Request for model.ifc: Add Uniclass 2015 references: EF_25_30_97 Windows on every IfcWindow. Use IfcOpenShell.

First a look at what the model holds.

```python
import ifcopenshell

model = ifcopenshell.open("model.ifc")
print(model.schema)
print("classifications:", [c.Name for c in model.by_type("IfcClassification")])
for ifc_class in ("IfcDoor", "IfcRoof", "IfcStair", "IfcWall", "IfcWindow"):
    print(ifc_class, len(model.by_type(ifc_class)))
```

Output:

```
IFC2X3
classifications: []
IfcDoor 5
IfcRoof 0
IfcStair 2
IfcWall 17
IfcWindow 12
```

```python
import ifcopenshell
import ifcopenshell.api.classification

model = ifcopenshell.open("model.ifc")

# IFC2X3 requires Source and Edition and has no link from the project to the system.
system = model.create_entity("IfcClassification", Source="NBS", Edition="2015", Name="Uniclass 2015")

codes = {
    "IfcWindow": ("EF_25_30_97", "Windows"),
}
for ifc_class, (code, name) in codes.items():
    products = model.by_type(ifc_class)
    ifcopenshell.api.classification.add_reference(
        model, products=products, classification=system, identification=code, name=name
    )
    print(code, len(products))

model.write("model_edited.ifc")
```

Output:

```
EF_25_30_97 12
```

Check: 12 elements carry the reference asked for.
